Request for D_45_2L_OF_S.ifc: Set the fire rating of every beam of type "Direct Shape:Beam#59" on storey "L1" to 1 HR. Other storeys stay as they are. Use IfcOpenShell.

First a look at what the model holds.

```python
import ifcopenshell
import ifcopenshell.util.element

model = ifcopenshell.open("D_45_2L_OF_S.ifc")
print(model.schema)
storey = next(s for s in model.by_type("IfcBuildingStorey") if s.Name == "L1")
beams = [e for e in ifcopenshell.util.element.get_decomposition(storey) if e.is_a("IfcBeam")]
seen = {}
for e in beams:
    element_type = ifcopenshell.util.element.get_type(e)
    key = (element_type.Name if element_type != e and element_type else None, ifcopenshell.util.element.get_pset(e, "Pset_BeamCommon", "FireRating"))
    seen[key] = seen.get(key, 0) + 1
for (name, value), count in sorted(seen.items(), key=str):
    print(count, "x", name, "|", value)
```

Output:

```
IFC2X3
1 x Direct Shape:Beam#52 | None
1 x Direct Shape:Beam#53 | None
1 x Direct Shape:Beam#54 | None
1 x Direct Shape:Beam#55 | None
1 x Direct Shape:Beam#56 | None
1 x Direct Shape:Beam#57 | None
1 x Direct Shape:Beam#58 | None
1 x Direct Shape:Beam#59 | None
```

```python
import ifcopenshell
import ifcopenshell.api.pset
import ifcopenshell.util.element

model = ifcopenshell.open("D_45_2L_OF_S.ifc")

storey = next(s for s in model.by_type("IfcBuildingStorey") if s.Name == "L1")
beams = [e for e in ifcopenshell.util.element.get_decomposition(storey) if e.is_a("IfcBeam")]

count = 0
for e in beams:
    element_type = ifcopenshell.util.element.get_type(e)
    if element_type in (None, e) or element_type.Name != "Direct Shape:Beam#59":
        continue
    # add_pset returns the element's existing set when there is one.
    pset = ifcopenshell.api.pset.add_pset(model, product=e, name="Pset_BeamCommon")
    ifcopenshell.api.pset.edit_pset(model, pset=pset, properties={"FireRating": "1 HR"})
    count += 1

print(count, "beams updated")

model.write("D_45_2L_OF_S-out.ifc")
```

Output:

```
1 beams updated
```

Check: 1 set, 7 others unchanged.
